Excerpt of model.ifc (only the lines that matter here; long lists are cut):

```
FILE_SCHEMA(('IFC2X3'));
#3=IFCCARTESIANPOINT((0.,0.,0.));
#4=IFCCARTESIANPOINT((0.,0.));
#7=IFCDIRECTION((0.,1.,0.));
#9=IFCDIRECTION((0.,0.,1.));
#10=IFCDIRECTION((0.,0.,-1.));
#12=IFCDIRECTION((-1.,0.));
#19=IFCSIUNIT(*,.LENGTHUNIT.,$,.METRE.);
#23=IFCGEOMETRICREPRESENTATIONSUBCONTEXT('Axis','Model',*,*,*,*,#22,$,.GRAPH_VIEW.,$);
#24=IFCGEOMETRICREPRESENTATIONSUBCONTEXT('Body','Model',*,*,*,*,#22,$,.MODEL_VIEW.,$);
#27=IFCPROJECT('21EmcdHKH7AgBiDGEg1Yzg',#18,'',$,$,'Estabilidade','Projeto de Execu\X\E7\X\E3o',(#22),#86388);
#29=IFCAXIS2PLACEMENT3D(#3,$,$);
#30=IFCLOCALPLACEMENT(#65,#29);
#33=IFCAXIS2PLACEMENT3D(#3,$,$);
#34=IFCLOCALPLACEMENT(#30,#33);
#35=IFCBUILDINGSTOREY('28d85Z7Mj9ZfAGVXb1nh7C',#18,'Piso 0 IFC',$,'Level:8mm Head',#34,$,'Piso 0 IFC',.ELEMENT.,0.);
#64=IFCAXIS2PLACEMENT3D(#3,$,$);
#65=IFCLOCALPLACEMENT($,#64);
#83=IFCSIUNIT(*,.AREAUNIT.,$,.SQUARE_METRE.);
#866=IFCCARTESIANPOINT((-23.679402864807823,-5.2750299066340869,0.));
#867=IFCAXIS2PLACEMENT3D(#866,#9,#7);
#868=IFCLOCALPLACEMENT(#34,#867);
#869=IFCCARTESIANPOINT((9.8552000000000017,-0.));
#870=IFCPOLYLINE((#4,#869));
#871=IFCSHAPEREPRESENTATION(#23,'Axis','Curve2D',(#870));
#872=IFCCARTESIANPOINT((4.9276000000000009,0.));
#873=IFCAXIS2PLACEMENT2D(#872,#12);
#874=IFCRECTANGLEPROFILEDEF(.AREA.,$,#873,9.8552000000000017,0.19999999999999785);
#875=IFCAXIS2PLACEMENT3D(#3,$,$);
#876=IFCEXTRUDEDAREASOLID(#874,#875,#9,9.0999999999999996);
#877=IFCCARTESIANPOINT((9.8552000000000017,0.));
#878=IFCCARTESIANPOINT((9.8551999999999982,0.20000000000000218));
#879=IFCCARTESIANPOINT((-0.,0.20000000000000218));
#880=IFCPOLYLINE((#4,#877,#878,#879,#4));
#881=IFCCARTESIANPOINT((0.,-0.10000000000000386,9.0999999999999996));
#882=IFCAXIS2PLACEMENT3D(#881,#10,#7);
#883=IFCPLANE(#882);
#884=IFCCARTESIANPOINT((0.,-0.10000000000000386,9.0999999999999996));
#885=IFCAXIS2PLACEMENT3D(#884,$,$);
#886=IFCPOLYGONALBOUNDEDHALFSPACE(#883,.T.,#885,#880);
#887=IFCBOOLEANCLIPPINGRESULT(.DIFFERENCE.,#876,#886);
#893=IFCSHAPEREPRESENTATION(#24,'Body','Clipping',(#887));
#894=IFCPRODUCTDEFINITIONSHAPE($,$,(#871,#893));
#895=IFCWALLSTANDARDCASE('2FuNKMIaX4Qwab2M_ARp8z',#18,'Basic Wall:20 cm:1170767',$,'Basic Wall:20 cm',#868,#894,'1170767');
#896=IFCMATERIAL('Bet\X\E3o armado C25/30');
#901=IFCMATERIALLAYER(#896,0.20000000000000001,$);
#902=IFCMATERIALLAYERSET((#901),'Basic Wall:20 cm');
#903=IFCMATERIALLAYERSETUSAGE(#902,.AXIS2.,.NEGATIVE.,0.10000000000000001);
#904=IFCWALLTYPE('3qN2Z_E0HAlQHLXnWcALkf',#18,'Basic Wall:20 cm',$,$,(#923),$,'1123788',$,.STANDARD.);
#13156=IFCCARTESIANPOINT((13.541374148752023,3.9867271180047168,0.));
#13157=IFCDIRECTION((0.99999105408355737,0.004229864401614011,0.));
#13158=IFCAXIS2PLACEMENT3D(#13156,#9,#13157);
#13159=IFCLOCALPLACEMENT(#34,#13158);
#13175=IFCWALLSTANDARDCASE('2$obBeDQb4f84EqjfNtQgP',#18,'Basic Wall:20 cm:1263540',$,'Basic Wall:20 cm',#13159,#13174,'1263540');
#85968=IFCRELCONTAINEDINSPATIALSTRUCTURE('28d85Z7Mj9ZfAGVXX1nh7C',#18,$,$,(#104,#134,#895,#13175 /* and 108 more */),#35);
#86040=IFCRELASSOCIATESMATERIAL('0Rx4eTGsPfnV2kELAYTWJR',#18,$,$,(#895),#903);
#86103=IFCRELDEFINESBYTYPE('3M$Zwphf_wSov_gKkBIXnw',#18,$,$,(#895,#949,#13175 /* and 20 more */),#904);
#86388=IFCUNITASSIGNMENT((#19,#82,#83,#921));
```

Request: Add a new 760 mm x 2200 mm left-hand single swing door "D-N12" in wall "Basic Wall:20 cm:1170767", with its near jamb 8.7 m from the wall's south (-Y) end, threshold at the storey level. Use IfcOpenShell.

```python
import numpy as np
import ifcopenshell
import ifcopenshell.api.feature
import ifcopenshell.api.geometry
import ifcopenshell.api.root
import ifcopenshell.api.spatial
import ifcopenshell.api.type
import ifcopenshell.geom
import ifcopenshell.util.element
import ifcopenshell.util.placement
import ifcopenshell.util.representation
import ifcopenshell.util.shape
import ifcopenshell.util.unit

model = ifcopenshell.open("model.ifc")
unit_scale = ifcopenshell.util.unit.calculate_unit_scale(model)
settings = ifcopenshell.geom.settings()


def volume(element):
    """Net volume in cubic metres, openings subtracted."""
    shape = ifcopenshell.geom.create_shape(settings, element)
    return ifcopenshell.util.shape.get_volume(shape.geometry)


wall = model.by_id(895)
storey = ifcopenshell.util.element.get_container(wall, ifc_class="IfcBuildingStorey")
context = ifcopenshell.util.representation.get_context(model, "Model", "Body", "MODEL_VIEW")
before = volume(wall)

width, height, from_end, sill = 0.76, 2.2, 8.7, 0.0  # metres

# The wall runs along its own X axis, and the end named is its -X end.
wall_shape = ifcopenshell.geom.create_shape(settings, wall)
x, y, z = ifcopenshell.util.shape.get_vertices(wall_shape.geometry).T
start = x.min() + from_end
face, thickness = float(y.min()), float(y.max() - y.min())
wall_matrix = ifcopenshell.util.placement.get_local_placement(wall.ObjectPlacement)
level = ifcopenshell.util.placement.get_local_placement(storey.ObjectPlacement)[2, 3]


def in_wall(x, y):
    """Placement at x, y metres in the wall's axes, at sill height."""
    matrix = wall_matrix.copy()
    matrix[:, 3] = wall_matrix @ np.array([x / unit_scale, y / unit_scale, 0.0, 1.0])
    matrix[2, 3] = level + sill / unit_scale
    return matrix


# Opening: a box that overshoots both wall faces by 50 mm.
opening = ifcopenshell.api.root.create_entity(model, ifc_class="IfcOpeningElement")
box = ifcopenshell.api.geometry.add_wall_representation(
    model, context=context, length=width, height=height, thickness=thickness + 0.1
)
ifcopenshell.api.geometry.assign_representation(model, product=opening, representation=box)
ifcopenshell.api.geometry.edit_object_placement(model, product=opening, matrix=in_wall(start, face - 0.05), is_si=False)
ifcopenshell.api.feature.add_feature(model, feature=opening, element=wall)

door = ifcopenshell.api.root.create_entity(model, ifc_class="IfcDoor", name="D-N12")
door.OverallWidth, door.OverallHeight = width / unit_scale, height / unit_scale
body = ifcopenshell.api.geometry.add_door_representation(
    model,
    context=context,
    overall_width=door.OverallWidth,
    overall_height=door.OverallHeight,
    operation_type="SINGLE_SWING_LEFT",
    lining_properties={"LiningDepth": thickness / unit_scale, "ThresholdDepth": thickness / unit_scale},
)
ifcopenshell.api.geometry.assign_representation(model, product=door, representation=body)
ifcopenshell.api.spatial.assign_container(model, products=[door], relating_structure=storey)
fills = ifcopenshell.api.feature.add_filling(model, opening=opening, element=door)
fills.OwnerHistory = door.OwnerHistory  # required in IFC2X3

# IFC2X3 keeps the operation on the door style.
style = ifcopenshell.api.root.create_entity(model, ifc_class="IfcDoorStyle", name="D-N12")
style.OperationType, style.ConstructionType = "SINGLE_SWING_LEFT", "NOTDEFINED"
style.ParameterTakesPrecedence = style.Sizeable = False
ifcopenshell.api.type.assign_type(model, related_objects=[door], relating_type=style)

# The lining spans the wall, so the door starts at the wall face.
ifcopenshell.api.geometry.edit_object_placement(model, product=door, matrix=in_wall(start, face), is_si=False)

after = volume(wall)

print(f"wall volume {before:.3f} -> {after:.3f} m3")

model.write("model-out.ifc")
```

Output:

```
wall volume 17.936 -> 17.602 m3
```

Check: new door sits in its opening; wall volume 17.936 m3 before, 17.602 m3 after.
